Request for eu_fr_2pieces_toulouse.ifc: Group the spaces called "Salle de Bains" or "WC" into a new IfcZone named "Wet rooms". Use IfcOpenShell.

First a look at what the model holds.

```python
import ifcopenshell

model = ifcopenshell.open("eu_fr_2pieces_toulouse.ifc")
print(model.schema)
seen = {}
for space in model.by_type("IfcSpace"):
    seen[space.LongName] = seen.get(space.LongName, 0) + 1
for name, count in sorted(seen.items(), key=str):
    print(count, "x", name)
print("zones:", [z.Name for z in model.by_type("IfcZone")][:20])
```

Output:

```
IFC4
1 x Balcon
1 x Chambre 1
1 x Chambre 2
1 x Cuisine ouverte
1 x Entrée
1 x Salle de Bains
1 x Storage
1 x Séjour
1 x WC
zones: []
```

```python
import ifcopenshell
import ifcopenshell.api.group
import ifcopenshell.api.root

model = ifcopenshell.open("eu_fr_2pieces_toulouse.ifc")

names = {"Salle de Bains", "WC"}
spaces = [s for s in model.by_type("IfcSpace") if s.LongName in names]

zone = ifcopenshell.api.root.create_entity(model, ifc_class="IfcZone", name="Wet rooms")
ifcopenshell.api.group.assign_group(model, products=spaces, group=zone)
print(len(spaces), "spaces in", zone.Name)

model.write("eu_fr_2pieces_toulouse_edited.ifc")
```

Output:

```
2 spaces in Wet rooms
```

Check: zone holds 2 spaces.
